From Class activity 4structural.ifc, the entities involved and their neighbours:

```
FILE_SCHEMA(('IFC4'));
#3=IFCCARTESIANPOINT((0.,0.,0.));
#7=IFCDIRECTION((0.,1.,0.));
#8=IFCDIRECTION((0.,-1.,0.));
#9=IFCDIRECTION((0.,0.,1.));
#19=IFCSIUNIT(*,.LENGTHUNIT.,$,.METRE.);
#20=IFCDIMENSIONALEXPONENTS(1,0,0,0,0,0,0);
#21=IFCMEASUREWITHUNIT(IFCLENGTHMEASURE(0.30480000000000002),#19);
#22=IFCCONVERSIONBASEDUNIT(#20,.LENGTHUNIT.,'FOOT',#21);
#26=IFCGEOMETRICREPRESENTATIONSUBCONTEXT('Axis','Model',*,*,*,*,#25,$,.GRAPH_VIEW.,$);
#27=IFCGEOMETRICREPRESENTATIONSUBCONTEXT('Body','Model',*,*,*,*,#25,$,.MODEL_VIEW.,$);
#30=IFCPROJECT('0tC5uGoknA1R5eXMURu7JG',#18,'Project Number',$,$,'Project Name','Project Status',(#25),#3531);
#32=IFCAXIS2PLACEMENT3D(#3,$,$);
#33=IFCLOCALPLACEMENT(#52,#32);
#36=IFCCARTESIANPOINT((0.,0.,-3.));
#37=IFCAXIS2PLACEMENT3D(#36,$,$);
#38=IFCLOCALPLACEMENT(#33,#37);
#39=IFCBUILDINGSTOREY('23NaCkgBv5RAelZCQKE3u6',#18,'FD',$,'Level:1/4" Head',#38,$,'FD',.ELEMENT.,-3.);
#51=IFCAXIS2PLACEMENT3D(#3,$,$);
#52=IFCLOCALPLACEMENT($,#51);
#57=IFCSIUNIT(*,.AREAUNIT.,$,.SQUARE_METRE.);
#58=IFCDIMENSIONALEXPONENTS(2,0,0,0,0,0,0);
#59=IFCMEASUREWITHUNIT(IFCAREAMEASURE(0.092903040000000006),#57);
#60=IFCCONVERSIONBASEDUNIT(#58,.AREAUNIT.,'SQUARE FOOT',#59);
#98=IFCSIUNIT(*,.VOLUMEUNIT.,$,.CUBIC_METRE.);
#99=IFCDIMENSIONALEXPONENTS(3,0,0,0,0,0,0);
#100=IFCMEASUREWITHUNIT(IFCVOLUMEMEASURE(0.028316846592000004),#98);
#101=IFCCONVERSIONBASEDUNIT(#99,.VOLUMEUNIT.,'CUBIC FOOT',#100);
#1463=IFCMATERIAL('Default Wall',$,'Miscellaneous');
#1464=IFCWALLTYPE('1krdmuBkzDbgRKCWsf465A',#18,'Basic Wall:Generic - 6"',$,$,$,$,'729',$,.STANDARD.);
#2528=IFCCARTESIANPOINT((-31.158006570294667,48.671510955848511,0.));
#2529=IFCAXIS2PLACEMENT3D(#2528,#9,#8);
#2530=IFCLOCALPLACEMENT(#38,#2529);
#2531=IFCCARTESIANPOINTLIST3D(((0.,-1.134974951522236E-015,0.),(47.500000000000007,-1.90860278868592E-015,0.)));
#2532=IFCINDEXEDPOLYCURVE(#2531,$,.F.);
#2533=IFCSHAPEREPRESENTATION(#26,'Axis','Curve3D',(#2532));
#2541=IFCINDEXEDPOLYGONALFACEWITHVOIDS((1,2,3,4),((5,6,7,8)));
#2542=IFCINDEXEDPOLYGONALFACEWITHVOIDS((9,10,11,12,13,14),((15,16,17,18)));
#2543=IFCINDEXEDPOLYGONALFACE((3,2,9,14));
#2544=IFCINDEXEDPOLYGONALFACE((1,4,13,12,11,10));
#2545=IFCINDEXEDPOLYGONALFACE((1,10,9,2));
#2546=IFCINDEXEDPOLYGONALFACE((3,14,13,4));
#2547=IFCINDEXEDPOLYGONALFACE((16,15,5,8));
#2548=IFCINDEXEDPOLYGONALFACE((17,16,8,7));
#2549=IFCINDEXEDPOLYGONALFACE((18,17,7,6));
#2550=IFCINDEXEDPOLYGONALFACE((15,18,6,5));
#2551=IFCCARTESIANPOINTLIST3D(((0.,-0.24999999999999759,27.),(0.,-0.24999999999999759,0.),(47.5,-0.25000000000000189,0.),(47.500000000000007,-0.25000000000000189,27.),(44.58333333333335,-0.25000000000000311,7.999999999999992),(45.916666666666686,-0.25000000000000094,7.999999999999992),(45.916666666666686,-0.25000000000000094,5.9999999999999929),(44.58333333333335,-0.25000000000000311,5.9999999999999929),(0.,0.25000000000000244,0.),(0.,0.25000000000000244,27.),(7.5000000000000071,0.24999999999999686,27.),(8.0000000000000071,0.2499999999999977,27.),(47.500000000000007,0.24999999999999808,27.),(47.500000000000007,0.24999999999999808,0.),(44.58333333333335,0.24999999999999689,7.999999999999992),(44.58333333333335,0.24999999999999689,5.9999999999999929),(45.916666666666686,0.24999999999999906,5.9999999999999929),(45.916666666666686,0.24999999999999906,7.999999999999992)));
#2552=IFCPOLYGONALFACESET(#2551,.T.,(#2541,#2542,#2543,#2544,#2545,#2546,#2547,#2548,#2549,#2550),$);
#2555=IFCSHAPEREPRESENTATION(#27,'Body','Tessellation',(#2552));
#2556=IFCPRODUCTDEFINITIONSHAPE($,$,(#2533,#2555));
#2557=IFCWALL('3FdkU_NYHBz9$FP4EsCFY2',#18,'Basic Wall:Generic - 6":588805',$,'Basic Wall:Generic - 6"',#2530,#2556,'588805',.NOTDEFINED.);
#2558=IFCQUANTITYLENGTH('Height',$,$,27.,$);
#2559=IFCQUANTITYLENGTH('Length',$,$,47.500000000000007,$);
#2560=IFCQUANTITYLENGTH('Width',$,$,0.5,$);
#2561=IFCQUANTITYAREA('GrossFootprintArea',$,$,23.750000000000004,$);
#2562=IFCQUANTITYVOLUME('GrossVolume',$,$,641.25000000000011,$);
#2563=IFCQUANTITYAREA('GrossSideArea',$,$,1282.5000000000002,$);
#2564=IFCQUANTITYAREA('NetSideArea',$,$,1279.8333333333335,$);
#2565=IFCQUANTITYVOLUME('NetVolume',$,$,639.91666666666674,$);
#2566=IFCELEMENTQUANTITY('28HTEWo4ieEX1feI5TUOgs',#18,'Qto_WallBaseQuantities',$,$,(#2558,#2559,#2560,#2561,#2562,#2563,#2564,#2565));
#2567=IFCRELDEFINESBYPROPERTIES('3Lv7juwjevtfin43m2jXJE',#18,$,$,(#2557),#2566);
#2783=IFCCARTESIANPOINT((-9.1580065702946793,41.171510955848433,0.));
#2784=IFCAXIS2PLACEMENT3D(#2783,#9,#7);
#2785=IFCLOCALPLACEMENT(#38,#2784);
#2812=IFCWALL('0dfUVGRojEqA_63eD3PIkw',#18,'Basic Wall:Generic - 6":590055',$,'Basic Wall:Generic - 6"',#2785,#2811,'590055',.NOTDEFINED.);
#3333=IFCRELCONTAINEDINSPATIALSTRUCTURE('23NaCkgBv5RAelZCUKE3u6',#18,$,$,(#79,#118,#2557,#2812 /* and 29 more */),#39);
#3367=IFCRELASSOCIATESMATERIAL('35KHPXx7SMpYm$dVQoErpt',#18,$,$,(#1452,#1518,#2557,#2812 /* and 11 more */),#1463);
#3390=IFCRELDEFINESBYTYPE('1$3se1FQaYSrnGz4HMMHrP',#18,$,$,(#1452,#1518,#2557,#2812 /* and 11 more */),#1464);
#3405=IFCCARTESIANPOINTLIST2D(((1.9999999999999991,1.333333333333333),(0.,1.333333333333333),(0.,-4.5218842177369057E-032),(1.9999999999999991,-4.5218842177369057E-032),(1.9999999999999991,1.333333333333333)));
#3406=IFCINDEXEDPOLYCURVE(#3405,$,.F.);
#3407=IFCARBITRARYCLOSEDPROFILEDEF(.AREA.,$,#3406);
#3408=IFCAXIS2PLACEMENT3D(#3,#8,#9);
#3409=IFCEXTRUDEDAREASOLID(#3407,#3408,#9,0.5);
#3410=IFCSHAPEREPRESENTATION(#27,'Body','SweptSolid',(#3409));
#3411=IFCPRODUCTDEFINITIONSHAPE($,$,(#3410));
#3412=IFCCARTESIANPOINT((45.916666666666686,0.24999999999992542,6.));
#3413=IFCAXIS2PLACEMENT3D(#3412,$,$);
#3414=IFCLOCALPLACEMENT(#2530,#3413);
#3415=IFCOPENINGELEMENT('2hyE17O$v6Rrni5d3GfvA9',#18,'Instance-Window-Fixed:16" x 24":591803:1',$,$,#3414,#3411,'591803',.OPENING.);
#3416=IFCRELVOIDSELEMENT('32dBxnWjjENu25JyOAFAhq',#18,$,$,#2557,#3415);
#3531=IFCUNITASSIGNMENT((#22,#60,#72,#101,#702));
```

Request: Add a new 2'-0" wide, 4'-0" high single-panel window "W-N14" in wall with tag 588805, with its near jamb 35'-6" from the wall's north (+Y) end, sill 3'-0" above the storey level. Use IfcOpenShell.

```python
import numpy as np
import ifcopenshell
import ifcopenshell.api.feature
import ifcopenshell.api.geometry
import ifcopenshell.api.pset
import ifcopenshell.api.root
import ifcopenshell.api.spatial
import ifcopenshell.geom
import ifcopenshell.util.element
import ifcopenshell.util.placement
import ifcopenshell.util.representation
import ifcopenshell.util.shape
import ifcopenshell.util.unit

model = ifcopenshell.open("Class activity 4structural.ifc")
unit_scale = ifcopenshell.util.unit.calculate_unit_scale(model)
area_scale = ifcopenshell.util.unit.calculate_unit_scale(model, "AREAUNIT")
volume_scale = ifcopenshell.util.unit.calculate_unit_scale(model, "VOLUMEUNIT")
settings = ifcopenshell.geom.settings()


def volume(element):
    """Net volume in cubic metres, openings subtracted."""
    shape = ifcopenshell.geom.create_shape(settings, element)
    return ifcopenshell.util.shape.get_volume(shape.geometry)


wall = model.by_guid("3FdkU_NYHBz9$FP4EsCFY2")
storey = ifcopenshell.util.element.get_container(wall, ifc_class="IfcBuildingStorey")
context = ifcopenshell.util.representation.get_context(model, "Model", "Body", "MODEL_VIEW")
before = volume(wall)

width, height, from_end, sill = 0.6096, 1.2192, 10.8204, 0.9144  # metres

# The wall runs along its own X axis, and the end named is its -X end.
wall_shape = ifcopenshell.geom.create_shape(settings, wall)
x, y, z = ifcopenshell.util.shape.get_vertices(wall_shape.geometry).T
start = x.min() + from_end
face, thickness = float(y.min()), float(y.max() - y.min())
wall_matrix = ifcopenshell.util.placement.get_local_placement(wall.ObjectPlacement)
level = ifcopenshell.util.placement.get_local_placement(storey.ObjectPlacement)[2, 3]


def in_wall(x, y):
    """Placement at x, y metres in the wall's axes, at sill height."""
    matrix = wall_matrix.copy()
    matrix[:, 3] = wall_matrix @ np.array([x / unit_scale, y / unit_scale, 0.0, 1.0])
    matrix[2, 3] = level + sill / unit_scale
    return matrix


# Opening: a box that overshoots both wall faces by 50 mm.
opening = ifcopenshell.api.root.create_entity(model, ifc_class="IfcOpeningElement", predefined_type="OPENING")
box = ifcopenshell.api.geometry.add_wall_representation(
    model, context=context, length=width, height=height, thickness=thickness + 0.1
)
ifcopenshell.api.geometry.assign_representation(model, product=opening, representation=box)
ifcopenshell.api.geometry.edit_object_placement(model, product=opening, matrix=in_wall(start, face - 0.05), is_si=False)
ifcopenshell.api.feature.add_feature(model, feature=opening, element=wall)

window = ifcopenshell.api.root.create_entity(model, ifc_class="IfcWindow", name="W-N14", predefined_type="WINDOW")
window.OverallWidth, window.OverallHeight = width / unit_scale, height / unit_scale
window.PartitioningType = "SINGLE_PANEL"
body = ifcopenshell.api.geometry.add_window_representation(
    model,
    context=context,
    overall_width=window.OverallWidth,
    overall_height=window.OverallHeight,
    partition_type="SINGLE_PANEL",
)
ifcopenshell.api.geometry.assign_representation(model, product=window, representation=body)
ifcopenshell.api.spatial.assign_container(model, products=[window], relating_structure=storey)
ifcopenshell.api.feature.add_filling(model, opening=opening, element=window)

# Centre the window in the wall's thickness.
ifcopenshell.api.geometry.edit_object_placement(model, product=window, matrix=in_wall(start, face), is_si=False)
window_shape = ifcopenshell.geom.create_shape(settings, window)
depth = ifcopenshell.util.shape.get_vertices(window_shape.geometry)[:, 1]
offset = face + thickness / 2 - (depth.min() + depth.max()) / 2
ifcopenshell.api.geometry.edit_object_placement(model, product=window, matrix=in_wall(start, offset), is_si=False)

after = volume(wall)

# Update the wall's stored quantities.
qto = model.by_id(ifcopenshell.util.element.get_pset(wall, "Qto_WallBaseQuantities", should_inherit=False)["id"])
ifcopenshell.api.pset.edit_qto(model, qto=qto, properties={
    "NetSideArea": after / thickness / area_scale,
    "NetVolume": after / volume_scale,
})

print(f"wall volume {before:.3f} -> {after:.3f} m3")

model.write("Class activity 4structural-out.ifc")
```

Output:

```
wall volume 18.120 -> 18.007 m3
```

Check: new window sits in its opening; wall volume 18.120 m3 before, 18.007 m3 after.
